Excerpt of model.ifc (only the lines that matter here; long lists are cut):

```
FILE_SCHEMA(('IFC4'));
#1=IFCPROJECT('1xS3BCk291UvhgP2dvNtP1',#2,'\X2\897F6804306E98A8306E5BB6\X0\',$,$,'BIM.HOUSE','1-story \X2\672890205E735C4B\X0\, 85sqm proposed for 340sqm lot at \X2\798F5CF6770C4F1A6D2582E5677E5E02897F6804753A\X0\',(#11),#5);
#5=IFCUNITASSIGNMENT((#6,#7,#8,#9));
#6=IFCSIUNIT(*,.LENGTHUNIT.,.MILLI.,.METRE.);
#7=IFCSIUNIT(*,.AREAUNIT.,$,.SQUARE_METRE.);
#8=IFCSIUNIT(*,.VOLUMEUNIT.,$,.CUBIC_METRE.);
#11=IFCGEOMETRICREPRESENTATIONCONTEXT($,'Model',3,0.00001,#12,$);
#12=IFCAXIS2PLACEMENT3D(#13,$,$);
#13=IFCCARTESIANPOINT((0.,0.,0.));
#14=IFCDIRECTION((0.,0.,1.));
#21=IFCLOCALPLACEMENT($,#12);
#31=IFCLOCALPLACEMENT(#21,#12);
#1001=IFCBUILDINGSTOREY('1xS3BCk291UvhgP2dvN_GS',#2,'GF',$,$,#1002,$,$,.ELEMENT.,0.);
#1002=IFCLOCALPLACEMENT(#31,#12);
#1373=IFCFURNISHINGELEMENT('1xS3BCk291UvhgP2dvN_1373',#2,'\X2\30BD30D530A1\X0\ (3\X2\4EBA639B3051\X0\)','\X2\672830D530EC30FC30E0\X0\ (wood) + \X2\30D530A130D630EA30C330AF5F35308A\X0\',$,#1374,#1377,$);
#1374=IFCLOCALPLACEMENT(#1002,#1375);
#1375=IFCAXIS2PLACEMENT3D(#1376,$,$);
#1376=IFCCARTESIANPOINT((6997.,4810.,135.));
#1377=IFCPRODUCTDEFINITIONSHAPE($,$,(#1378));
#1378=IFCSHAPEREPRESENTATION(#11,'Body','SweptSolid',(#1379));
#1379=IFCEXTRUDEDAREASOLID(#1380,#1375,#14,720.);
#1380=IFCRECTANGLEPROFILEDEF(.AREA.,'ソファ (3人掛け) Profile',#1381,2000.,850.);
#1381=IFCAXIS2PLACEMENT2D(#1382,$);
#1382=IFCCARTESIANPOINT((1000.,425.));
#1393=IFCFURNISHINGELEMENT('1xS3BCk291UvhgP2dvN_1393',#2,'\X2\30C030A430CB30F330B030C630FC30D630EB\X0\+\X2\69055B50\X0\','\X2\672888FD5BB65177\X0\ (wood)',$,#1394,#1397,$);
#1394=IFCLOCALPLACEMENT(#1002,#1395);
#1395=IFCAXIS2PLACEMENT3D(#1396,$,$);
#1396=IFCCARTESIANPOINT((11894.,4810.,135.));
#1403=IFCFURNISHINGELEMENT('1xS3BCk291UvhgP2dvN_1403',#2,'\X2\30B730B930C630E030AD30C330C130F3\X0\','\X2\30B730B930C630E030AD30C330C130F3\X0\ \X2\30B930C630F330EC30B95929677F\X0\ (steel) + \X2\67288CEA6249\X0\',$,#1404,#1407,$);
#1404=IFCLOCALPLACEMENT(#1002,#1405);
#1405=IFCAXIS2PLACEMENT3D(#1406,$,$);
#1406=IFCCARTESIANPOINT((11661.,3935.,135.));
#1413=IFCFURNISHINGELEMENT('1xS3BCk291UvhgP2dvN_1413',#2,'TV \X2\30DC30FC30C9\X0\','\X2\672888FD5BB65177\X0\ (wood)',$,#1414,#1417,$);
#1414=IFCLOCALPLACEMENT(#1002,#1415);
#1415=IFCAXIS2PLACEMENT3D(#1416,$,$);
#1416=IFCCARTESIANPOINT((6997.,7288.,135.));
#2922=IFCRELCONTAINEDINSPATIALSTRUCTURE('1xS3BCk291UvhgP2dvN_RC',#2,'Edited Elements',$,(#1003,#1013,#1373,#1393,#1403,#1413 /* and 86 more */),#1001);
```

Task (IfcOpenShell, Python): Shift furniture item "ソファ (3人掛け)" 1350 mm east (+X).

```python
import ifcopenshell
import ifcopenshell.api.geometry
import ifcopenshell.util.placement

model = ifcopenshell.open("model.ifc")

item = model.by_guid("1xS3BCk291UvhgP2dvN_1373")
matrix = ifcopenshell.util.placement.get_local_placement(item.ObjectPlacement)
matrix[0, 3] += 1350.0
ifcopenshell.api.geometry.edit_object_placement(model, product=item, matrix=matrix, is_si=False)

print(ifcopenshell.util.placement.get_local_placement(item.ObjectPlacement).round(3) + 0.0)

model.write("model_v2.ifc")
```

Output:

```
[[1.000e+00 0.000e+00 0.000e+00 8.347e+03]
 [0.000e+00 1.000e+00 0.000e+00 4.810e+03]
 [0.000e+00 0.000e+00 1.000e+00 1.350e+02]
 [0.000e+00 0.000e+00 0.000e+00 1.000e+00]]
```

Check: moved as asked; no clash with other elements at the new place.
